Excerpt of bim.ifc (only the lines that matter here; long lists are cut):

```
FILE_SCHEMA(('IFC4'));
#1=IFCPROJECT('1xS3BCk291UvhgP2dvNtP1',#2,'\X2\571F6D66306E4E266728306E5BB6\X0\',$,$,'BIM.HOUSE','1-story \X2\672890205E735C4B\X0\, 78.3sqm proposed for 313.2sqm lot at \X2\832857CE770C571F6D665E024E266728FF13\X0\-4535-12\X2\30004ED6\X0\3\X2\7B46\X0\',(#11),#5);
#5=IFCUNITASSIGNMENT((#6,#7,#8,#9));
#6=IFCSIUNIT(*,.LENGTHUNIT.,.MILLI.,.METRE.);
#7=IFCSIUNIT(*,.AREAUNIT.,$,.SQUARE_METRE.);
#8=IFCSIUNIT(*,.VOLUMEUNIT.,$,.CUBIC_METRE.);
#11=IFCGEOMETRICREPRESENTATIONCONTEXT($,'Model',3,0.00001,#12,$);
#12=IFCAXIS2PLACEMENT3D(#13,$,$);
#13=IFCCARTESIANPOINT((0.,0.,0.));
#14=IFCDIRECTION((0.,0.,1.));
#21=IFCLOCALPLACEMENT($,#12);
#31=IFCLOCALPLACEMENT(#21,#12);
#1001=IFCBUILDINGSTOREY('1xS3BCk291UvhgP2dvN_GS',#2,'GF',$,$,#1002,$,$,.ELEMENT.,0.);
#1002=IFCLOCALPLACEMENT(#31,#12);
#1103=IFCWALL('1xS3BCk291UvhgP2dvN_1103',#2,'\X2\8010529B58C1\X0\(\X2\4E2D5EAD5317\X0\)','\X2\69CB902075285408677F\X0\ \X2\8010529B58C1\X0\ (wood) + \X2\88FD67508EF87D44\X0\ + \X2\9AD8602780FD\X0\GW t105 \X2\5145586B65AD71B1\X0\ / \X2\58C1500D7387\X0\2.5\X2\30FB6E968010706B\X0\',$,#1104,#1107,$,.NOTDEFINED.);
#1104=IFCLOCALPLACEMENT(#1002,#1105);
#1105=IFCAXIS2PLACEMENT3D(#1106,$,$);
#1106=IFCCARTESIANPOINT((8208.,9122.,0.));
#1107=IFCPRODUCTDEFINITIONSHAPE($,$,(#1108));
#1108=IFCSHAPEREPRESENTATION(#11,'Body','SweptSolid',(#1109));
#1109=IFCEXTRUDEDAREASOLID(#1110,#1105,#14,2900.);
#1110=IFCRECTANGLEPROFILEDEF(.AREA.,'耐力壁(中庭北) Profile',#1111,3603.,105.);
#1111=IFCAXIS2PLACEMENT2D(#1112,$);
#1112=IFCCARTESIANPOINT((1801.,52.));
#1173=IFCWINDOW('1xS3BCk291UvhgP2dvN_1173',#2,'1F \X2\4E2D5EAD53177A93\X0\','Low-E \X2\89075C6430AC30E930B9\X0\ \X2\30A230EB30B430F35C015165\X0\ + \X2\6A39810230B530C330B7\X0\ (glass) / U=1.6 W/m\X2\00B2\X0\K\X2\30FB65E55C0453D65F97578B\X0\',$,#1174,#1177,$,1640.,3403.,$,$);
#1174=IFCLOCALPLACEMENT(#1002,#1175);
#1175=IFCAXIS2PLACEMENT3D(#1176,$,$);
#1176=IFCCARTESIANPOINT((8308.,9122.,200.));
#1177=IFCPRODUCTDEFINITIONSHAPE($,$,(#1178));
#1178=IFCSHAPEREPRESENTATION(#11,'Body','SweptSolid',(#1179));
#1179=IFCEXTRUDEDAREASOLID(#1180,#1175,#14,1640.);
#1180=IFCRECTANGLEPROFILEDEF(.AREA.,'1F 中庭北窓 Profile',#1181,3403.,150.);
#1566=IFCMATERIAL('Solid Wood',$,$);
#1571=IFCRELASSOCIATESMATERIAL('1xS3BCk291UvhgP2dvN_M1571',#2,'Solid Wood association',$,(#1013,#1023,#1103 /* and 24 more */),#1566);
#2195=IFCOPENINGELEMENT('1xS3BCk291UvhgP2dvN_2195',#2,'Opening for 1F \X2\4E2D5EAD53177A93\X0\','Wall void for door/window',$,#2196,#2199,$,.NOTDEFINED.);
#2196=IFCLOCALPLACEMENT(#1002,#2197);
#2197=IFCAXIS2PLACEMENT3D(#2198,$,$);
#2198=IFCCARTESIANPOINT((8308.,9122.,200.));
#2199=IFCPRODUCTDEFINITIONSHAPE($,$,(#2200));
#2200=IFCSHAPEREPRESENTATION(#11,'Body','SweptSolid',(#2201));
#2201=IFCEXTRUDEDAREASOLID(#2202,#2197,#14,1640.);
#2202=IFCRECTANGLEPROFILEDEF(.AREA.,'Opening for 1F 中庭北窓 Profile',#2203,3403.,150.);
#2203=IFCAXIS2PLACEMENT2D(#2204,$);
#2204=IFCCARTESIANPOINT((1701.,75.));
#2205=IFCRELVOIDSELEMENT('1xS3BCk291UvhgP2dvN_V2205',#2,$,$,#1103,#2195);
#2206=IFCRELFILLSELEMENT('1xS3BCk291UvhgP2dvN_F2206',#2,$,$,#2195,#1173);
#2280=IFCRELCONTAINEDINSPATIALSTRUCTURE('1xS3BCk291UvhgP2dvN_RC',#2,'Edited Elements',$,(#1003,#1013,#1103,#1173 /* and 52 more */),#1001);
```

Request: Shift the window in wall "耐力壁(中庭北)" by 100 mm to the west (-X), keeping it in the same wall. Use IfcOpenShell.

```python
import ifcopenshell
import ifcopenshell.api.geometry
import ifcopenshell.util.placement
import ifcopenshell.util.unit

model = ifcopenshell.open("bim.ifc")
unit_scale = ifcopenshell.util.unit.calculate_unit_scale(model)

window = model.by_id(1173)
opening = window.FillsVoids[0].RelatingOpeningElement
wall = opening.VoidsElements[0].RelatingBuildingElement

wall_matrix = ifcopenshell.util.placement.get_local_placement(wall.ObjectPlacement)
shift = wall_matrix[:3, 0] * -0.1 / unit_scale
before = ifcopenshell.util.placement.get_local_placement(window.ObjectPlacement)[:3, 3].copy()

# The window is not placed relative to its opening, so move both.
for product in (opening, window):
    matrix = ifcopenshell.util.placement.get_local_placement(product.ObjectPlacement)
    matrix[:3, 3] += shift
    ifcopenshell.api.geometry.edit_object_placement(model, product=product, matrix=matrix, is_si=False)

after = ifcopenshell.util.placement.get_local_placement(window.ObjectPlacement)[:3, 3]
print("window moved by", (after - before).round(3) + 0.0)

model.write("bim_rev.ifc")
```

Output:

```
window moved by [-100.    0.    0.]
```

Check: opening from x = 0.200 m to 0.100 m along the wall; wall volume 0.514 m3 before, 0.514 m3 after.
